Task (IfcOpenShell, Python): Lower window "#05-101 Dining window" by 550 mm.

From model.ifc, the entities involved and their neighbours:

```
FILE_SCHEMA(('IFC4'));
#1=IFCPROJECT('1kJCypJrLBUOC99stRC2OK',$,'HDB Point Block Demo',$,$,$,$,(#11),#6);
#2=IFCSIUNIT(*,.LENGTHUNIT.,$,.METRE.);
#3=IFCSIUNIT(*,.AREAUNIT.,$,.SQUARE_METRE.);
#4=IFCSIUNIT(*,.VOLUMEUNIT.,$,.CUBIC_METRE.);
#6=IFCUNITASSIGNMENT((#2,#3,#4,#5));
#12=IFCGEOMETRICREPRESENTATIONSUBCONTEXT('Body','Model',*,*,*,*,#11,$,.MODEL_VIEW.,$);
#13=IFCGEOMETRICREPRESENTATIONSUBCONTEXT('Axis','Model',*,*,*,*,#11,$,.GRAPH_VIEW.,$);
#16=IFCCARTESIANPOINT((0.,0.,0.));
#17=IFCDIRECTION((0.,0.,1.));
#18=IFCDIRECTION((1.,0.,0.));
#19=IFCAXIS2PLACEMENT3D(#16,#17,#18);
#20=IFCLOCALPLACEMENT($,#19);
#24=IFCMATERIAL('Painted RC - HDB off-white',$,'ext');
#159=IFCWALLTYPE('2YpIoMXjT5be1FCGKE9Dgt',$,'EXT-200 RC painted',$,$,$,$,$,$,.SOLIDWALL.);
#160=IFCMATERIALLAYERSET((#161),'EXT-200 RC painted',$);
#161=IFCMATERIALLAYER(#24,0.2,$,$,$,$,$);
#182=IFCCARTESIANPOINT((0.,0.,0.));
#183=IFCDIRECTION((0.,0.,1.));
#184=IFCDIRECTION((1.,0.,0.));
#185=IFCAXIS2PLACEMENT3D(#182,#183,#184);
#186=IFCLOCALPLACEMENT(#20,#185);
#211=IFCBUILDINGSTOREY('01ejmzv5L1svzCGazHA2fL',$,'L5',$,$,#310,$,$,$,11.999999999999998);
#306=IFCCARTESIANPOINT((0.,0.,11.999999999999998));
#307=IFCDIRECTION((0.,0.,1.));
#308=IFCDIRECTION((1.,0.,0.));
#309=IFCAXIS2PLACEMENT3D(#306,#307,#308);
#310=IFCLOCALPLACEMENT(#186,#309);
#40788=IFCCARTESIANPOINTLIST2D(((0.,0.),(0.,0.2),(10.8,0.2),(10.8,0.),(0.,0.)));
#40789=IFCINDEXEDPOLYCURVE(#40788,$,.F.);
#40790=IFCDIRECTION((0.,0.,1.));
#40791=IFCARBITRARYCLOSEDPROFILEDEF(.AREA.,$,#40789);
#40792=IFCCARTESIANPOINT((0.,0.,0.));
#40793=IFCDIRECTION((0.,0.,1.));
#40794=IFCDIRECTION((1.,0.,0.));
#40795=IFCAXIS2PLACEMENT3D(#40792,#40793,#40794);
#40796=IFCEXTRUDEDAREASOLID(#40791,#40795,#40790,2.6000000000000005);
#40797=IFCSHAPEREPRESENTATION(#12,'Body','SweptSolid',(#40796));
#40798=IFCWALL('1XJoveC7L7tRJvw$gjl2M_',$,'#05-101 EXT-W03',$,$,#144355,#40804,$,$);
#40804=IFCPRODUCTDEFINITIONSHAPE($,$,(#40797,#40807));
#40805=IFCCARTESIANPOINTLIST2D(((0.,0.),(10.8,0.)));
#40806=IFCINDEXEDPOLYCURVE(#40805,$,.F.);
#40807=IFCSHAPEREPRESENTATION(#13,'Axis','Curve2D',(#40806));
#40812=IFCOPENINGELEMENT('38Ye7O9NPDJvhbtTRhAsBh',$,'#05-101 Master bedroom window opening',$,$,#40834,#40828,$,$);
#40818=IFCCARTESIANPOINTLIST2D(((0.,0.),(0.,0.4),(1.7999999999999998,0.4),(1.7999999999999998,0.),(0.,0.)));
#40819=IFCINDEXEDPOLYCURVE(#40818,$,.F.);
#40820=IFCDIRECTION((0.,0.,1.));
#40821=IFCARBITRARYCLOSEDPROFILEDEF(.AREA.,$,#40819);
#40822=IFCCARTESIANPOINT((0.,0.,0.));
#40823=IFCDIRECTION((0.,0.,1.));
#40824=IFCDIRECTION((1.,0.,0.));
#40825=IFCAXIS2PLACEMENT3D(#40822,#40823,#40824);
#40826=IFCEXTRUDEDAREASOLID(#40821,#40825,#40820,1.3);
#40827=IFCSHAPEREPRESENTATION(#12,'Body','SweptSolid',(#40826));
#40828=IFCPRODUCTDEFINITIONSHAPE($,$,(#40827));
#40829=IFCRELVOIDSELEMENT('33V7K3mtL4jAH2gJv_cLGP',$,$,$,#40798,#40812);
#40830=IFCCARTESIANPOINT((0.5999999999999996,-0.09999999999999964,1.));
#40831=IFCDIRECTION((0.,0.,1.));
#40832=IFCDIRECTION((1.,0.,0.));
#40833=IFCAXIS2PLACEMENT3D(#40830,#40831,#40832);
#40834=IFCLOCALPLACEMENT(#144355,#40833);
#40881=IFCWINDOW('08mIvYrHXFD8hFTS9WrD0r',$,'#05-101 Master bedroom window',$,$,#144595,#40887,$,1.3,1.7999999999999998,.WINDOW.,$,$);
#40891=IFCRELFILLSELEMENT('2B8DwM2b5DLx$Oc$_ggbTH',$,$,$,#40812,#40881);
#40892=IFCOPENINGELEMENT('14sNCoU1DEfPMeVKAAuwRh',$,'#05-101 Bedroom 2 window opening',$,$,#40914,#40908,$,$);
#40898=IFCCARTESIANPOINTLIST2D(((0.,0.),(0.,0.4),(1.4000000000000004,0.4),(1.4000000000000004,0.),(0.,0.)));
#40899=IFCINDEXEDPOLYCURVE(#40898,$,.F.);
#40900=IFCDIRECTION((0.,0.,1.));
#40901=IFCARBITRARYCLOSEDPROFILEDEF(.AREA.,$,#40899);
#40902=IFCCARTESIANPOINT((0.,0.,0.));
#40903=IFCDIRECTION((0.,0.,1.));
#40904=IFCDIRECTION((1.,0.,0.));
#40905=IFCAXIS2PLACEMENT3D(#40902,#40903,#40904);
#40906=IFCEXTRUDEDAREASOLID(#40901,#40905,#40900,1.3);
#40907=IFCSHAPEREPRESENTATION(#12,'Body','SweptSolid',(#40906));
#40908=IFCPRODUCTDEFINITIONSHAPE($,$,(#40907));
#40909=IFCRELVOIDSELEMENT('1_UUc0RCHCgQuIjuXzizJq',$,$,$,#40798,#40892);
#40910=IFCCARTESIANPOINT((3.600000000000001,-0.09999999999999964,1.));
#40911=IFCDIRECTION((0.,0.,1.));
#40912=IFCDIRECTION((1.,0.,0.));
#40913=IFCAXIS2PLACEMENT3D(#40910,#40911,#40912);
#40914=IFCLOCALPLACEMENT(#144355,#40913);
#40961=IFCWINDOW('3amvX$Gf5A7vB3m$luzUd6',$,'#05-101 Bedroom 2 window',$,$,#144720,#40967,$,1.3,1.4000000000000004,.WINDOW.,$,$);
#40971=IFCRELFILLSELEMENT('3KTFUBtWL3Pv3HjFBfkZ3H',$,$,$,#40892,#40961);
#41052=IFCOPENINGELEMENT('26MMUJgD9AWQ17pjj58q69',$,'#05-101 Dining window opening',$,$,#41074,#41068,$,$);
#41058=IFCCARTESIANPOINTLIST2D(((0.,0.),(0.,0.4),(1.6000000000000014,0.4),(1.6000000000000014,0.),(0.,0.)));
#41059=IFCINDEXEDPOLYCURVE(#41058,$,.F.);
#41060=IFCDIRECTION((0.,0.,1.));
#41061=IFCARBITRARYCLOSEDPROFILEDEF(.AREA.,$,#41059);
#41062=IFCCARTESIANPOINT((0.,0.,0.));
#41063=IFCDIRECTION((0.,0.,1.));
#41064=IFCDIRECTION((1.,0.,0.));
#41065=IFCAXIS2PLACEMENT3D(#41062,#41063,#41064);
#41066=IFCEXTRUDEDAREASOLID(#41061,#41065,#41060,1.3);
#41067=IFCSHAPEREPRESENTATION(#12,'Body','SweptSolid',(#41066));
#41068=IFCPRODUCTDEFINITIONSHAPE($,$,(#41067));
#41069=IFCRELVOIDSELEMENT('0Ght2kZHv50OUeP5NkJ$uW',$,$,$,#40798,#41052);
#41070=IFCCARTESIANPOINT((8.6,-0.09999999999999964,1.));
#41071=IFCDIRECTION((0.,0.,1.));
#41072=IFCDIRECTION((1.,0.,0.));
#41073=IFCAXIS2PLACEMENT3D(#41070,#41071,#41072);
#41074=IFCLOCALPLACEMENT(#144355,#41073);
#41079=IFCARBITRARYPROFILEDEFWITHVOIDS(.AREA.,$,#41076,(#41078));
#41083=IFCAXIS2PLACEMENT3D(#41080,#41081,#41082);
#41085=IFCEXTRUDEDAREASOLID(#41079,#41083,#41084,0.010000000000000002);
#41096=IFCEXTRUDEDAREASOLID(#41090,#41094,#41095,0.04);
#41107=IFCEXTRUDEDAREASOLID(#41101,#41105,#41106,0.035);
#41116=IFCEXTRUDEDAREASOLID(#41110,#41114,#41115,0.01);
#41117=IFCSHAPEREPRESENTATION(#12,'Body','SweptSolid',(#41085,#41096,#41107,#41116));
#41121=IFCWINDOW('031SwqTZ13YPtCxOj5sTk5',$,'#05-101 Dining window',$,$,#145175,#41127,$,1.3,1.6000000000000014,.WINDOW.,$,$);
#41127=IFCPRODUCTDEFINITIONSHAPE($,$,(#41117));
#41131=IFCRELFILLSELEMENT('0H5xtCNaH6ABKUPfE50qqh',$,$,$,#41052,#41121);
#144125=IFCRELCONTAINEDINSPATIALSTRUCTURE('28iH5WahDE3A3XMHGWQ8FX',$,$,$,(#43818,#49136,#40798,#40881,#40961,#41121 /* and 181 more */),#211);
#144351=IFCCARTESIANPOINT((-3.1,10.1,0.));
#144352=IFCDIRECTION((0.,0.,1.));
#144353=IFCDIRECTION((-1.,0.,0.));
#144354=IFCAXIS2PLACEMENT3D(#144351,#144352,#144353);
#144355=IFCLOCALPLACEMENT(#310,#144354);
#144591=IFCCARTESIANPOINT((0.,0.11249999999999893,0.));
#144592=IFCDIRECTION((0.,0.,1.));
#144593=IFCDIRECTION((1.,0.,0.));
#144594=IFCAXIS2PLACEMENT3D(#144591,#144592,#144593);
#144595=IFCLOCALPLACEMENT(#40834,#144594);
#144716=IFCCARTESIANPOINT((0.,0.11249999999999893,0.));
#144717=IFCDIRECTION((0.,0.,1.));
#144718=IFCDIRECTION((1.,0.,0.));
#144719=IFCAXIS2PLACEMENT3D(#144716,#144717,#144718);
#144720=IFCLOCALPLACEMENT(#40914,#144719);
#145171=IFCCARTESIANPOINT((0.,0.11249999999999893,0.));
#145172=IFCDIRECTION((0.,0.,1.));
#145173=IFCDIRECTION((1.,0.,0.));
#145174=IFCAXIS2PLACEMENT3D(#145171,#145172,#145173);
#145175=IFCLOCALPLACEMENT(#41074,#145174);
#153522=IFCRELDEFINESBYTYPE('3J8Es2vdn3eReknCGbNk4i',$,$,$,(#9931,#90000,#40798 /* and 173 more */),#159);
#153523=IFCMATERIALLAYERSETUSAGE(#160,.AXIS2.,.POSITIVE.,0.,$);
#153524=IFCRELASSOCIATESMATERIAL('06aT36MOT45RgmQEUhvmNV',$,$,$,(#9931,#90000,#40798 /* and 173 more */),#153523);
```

```python
import numpy as np
import ifcopenshell
import ifcopenshell.api.geometry
import ifcopenshell.util.placement
import ifcopenshell.util.unit

model = ifcopenshell.open("model.ifc")
unit_scale = ifcopenshell.util.unit.calculate_unit_scale(model)

window = model.by_guid("031SwqTZ13YPtCxOj5sTk5")
opening = window.FillsVoids[0].RelatingOpeningElement
dz = -0.55 / unit_scale

shift = np.array([0.0, 0.0, dz])
# The window is placed relative to its opening, so it follows when the opening moves.
matrix = ifcopenshell.util.placement.get_local_placement(opening.ObjectPlacement)
matrix[:3, 3] += shift
ifcopenshell.api.geometry.edit_object_placement(
    model, product=opening, matrix=matrix, is_si=False, should_transform_children=True
)

print(f"moved by {dz * unit_scale:+.3f} m")

model.write("model_edited.ifc")
```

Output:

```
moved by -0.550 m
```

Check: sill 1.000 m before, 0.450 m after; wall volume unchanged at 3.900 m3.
